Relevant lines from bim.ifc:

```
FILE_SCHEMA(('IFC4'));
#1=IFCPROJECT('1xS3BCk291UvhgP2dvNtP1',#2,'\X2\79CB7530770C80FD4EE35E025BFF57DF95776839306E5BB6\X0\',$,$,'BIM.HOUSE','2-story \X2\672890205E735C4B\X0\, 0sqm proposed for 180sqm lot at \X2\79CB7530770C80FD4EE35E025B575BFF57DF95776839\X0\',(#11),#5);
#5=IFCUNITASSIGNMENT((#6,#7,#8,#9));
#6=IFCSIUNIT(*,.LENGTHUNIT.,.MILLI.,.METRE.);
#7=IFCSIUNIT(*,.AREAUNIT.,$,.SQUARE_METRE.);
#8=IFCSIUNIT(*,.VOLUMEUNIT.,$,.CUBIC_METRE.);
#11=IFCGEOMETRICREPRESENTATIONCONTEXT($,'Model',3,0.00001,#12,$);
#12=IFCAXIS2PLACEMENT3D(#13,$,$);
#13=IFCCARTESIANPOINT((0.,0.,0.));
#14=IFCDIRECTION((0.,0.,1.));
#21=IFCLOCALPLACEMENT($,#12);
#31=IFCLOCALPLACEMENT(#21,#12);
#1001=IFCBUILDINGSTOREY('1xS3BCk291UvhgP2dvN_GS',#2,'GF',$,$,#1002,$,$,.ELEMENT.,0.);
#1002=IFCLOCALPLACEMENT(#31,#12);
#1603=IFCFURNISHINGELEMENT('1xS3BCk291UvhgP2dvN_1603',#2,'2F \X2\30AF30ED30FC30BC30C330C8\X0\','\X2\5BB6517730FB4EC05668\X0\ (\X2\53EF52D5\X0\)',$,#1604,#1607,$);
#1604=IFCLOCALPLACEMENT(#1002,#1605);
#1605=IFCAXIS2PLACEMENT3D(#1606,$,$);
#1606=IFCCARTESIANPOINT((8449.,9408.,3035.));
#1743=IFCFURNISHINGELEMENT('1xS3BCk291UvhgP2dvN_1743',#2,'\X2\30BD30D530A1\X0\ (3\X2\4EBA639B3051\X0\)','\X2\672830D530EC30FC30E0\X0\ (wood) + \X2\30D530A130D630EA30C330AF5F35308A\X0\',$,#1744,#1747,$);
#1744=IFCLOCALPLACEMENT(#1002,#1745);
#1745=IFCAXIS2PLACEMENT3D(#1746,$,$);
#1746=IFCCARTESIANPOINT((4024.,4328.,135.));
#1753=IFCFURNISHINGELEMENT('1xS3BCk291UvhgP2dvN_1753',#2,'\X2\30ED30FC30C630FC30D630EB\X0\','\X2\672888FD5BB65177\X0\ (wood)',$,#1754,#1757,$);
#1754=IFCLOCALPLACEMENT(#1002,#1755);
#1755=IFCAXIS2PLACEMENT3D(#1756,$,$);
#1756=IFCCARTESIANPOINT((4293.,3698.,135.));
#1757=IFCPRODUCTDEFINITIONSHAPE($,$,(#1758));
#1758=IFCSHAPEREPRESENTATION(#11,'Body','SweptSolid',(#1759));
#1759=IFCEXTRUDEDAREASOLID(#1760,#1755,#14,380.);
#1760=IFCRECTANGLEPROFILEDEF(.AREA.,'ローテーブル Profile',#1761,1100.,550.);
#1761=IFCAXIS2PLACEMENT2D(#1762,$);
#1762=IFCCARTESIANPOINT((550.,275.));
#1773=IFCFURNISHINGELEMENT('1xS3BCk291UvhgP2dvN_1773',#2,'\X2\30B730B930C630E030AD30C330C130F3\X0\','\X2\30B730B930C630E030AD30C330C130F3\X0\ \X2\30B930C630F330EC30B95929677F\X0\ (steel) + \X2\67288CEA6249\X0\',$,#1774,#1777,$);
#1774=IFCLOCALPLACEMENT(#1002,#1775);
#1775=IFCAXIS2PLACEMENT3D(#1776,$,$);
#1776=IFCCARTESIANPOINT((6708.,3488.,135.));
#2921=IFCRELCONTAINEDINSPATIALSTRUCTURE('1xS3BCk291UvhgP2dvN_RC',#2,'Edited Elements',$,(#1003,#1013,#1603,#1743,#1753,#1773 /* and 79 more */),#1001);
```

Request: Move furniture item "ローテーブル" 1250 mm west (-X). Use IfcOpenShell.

```python
import ifcopenshell
import ifcopenshell.api.geometry
import ifcopenshell.util.placement
import ifcopenshell.util.unit

model = ifcopenshell.open("bim.ifc")
unit_scale = ifcopenshell.util.unit.calculate_unit_scale(model)

item = model.by_guid("1xS3BCk291UvhgP2dvN_1753")
matrix = ifcopenshell.util.placement.get_local_placement(item.ObjectPlacement)
matrix[0, 3] -= 1.25 / unit_scale
ifcopenshell.api.geometry.edit_object_placement(model, product=item, matrix=matrix, is_si=False)

print(ifcopenshell.util.placement.get_local_placement(item.ObjectPlacement).round(3) + 0.0)

model.write("bim_v2.ifc")
```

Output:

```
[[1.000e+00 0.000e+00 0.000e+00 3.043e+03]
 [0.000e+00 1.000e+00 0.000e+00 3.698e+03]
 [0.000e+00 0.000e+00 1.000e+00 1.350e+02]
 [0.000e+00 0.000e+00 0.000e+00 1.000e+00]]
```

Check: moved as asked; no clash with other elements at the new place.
